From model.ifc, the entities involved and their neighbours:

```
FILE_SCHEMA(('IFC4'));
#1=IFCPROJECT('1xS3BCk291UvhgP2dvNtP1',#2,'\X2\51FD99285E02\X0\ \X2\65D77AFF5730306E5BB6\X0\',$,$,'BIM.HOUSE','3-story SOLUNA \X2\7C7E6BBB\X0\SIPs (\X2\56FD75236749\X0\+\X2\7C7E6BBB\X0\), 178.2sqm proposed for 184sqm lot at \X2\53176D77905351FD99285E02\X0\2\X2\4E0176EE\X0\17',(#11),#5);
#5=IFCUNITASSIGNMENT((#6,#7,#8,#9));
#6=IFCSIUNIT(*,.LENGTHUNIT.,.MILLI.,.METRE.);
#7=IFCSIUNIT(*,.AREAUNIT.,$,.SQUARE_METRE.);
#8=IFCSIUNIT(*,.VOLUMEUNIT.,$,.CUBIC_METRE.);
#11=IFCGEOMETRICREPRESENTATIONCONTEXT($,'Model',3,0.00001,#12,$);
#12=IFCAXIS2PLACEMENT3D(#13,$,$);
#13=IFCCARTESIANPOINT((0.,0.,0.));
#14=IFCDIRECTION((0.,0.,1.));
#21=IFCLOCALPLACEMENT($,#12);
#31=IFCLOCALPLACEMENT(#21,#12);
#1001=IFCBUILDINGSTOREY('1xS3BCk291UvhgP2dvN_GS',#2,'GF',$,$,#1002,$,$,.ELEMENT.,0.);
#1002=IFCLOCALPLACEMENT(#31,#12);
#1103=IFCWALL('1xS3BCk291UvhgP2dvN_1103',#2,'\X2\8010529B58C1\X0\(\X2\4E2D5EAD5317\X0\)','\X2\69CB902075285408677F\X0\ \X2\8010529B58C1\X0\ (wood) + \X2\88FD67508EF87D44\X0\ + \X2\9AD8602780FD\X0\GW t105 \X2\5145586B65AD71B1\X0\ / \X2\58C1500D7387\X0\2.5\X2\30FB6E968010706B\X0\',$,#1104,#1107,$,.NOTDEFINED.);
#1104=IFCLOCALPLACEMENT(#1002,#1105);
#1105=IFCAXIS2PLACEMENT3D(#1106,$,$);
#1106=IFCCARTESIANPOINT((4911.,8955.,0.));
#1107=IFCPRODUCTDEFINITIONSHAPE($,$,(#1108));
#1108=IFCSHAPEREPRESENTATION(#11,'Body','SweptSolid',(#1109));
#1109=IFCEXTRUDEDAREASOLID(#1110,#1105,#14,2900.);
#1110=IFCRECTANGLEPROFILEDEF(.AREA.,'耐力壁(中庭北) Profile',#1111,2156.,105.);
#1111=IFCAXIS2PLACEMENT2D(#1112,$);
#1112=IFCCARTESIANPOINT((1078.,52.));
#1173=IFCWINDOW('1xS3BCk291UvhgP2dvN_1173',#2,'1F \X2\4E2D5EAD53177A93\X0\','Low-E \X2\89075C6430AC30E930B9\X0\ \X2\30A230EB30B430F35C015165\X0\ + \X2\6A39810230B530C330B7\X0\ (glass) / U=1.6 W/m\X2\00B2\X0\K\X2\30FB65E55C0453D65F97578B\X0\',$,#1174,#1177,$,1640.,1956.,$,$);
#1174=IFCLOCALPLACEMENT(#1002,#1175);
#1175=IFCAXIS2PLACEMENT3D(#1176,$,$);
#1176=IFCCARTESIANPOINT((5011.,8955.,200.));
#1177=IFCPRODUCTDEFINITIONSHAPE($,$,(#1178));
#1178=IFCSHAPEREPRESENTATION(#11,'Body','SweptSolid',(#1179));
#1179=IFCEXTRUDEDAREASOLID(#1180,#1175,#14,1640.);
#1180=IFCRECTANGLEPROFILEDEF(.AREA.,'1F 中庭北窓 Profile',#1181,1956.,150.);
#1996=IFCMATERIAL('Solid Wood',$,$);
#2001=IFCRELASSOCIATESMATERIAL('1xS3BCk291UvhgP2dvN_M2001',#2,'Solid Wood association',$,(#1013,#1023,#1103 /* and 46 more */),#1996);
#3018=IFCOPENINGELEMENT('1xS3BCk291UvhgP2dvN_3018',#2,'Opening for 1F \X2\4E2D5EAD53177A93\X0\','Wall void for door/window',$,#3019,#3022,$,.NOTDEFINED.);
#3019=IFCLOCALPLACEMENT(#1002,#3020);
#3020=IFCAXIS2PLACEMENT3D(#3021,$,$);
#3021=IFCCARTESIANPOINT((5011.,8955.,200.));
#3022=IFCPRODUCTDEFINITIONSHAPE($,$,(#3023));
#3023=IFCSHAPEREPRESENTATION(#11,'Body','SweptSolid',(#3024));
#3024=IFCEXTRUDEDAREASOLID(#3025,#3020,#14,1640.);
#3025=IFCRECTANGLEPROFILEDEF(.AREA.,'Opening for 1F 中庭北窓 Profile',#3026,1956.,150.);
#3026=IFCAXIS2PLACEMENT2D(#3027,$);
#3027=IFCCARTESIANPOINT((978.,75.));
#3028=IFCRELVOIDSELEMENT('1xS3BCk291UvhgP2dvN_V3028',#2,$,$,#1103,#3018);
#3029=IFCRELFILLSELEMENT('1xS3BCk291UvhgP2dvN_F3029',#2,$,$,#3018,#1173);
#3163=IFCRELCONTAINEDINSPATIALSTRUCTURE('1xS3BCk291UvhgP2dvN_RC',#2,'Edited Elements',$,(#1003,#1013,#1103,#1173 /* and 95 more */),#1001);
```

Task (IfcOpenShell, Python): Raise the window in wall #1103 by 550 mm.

```python
import numpy as np
import ifcopenshell
import ifcopenshell.api.geometry
import ifcopenshell.util.placement
import ifcopenshell.util.unit

model = ifcopenshell.open("model.ifc")
unit_scale = ifcopenshell.util.unit.calculate_unit_scale(model)

window = model.by_guid("1xS3BCk291UvhgP2dvN_1173")
opening = window.FillsVoids[0].RelatingOpeningElement
dz = 550.0

shift = np.array([0.0, 0.0, dz])
# The window is not placed relative to its opening, so move both.
for product in (opening, window):
    matrix = ifcopenshell.util.placement.get_local_placement(product.ObjectPlacement)
    matrix[:3, 3] += shift
    ifcopenshell.api.geometry.edit_object_placement(model, product=product, matrix=matrix, is_si=False)

print(f"moved by {dz * unit_scale:+.3f} m")

model.write("model_rev.ifc")
```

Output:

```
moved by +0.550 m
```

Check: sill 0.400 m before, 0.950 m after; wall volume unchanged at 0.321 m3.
